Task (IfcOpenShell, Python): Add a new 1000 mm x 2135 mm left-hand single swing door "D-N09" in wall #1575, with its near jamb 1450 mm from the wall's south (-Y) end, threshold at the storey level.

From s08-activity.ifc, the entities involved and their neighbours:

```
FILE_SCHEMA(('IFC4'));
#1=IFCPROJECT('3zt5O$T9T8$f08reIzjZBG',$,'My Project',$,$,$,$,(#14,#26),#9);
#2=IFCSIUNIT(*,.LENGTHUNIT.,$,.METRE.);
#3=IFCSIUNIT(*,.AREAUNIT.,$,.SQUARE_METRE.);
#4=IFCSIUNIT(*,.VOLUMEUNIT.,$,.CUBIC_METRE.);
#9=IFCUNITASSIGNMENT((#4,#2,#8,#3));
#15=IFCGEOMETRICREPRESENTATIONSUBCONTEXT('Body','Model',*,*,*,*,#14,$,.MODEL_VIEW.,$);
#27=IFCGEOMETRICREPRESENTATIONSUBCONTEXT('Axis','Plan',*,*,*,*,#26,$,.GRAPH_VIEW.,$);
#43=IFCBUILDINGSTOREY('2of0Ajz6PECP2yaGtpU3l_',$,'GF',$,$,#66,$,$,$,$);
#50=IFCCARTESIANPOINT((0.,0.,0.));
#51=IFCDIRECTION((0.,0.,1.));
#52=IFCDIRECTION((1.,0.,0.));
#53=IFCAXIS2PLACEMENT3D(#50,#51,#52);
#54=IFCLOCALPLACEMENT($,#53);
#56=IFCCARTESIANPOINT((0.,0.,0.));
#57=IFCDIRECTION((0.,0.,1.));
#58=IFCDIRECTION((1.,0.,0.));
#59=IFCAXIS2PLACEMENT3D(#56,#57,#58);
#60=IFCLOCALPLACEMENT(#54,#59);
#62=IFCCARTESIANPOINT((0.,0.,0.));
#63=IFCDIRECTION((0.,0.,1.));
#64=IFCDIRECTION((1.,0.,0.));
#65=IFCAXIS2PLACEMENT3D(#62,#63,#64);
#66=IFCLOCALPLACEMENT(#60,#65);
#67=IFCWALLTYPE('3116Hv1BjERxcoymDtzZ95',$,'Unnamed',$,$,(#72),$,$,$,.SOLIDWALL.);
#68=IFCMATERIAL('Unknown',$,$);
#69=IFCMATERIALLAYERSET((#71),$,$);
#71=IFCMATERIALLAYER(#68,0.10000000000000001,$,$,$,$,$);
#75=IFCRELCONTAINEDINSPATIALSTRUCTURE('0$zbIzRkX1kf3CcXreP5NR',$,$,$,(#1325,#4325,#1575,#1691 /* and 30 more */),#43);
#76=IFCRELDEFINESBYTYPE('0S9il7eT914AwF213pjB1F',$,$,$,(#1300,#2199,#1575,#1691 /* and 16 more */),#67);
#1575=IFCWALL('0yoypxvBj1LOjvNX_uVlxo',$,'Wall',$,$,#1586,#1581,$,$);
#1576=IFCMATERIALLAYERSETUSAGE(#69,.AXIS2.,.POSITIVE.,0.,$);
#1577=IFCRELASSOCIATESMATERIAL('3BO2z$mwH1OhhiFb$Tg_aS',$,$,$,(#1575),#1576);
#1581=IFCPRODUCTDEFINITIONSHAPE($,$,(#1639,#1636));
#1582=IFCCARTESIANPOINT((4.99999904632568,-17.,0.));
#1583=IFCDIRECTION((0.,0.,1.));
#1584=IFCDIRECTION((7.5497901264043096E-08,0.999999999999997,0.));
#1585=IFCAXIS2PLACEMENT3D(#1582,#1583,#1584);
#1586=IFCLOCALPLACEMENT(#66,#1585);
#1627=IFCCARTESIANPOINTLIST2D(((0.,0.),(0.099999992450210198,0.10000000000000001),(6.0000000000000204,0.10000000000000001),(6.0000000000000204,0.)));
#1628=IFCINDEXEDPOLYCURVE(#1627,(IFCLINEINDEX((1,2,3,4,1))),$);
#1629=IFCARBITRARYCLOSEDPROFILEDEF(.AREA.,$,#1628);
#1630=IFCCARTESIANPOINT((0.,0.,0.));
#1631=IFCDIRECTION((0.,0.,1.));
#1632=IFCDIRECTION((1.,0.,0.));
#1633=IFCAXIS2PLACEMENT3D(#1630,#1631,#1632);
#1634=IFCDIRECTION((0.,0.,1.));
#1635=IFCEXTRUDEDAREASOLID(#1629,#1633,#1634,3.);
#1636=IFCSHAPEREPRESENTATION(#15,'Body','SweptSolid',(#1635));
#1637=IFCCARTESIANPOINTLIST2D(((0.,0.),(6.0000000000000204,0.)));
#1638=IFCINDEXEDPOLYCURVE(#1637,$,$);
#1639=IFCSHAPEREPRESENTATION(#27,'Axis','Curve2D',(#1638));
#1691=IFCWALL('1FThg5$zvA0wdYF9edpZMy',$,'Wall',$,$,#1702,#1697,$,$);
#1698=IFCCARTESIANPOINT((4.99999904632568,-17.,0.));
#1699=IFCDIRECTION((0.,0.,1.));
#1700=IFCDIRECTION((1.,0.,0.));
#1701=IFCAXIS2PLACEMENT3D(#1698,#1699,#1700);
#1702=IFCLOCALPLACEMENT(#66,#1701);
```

```python
import numpy as np
import ifcopenshell
import ifcopenshell.api.feature
import ifcopenshell.api.geometry
import ifcopenshell.api.root
import ifcopenshell.api.spatial
import ifcopenshell.geom
import ifcopenshell.util.element
import ifcopenshell.util.placement
import ifcopenshell.util.representation
import ifcopenshell.util.shape
import ifcopenshell.util.unit

model = ifcopenshell.open("s08-activity.ifc")
unit_scale = ifcopenshell.util.unit.calculate_unit_scale(model)
settings = ifcopenshell.geom.settings()


def volume(element):
    """Net volume in cubic metres, openings subtracted."""
    shape = ifcopenshell.geom.create_shape(settings, element)
    return ifcopenshell.util.shape.get_volume(shape.geometry)


wall = model.by_guid("0yoypxvBj1LOjvNX_uVlxo")
storey = ifcopenshell.util.element.get_container(wall, ifc_class="IfcBuildingStorey")
context = ifcopenshell.util.representation.get_context(model, "Model", "Body", "MODEL_VIEW")
before = volume(wall)

width, height, from_end, sill = 1, 2.135, 1.45, 0.0  # metres

# The wall runs along its own X axis, and the end named is its -X end.
wall_shape = ifcopenshell.geom.create_shape(settings, wall)
x, y, z = ifcopenshell.util.shape.get_vertices(wall_shape.geometry).T
start = x.min() + from_end
face, thickness = float(y.min()), float(y.max() - y.min())
wall_matrix = ifcopenshell.util.placement.get_local_placement(wall.ObjectPlacement)
level = ifcopenshell.util.placement.get_local_placement(storey.ObjectPlacement)[2, 3]


def in_wall(x, y):
    """Placement at x, y metres in the wall's axes, at sill height."""
    matrix = wall_matrix.copy()
    matrix[:, 3] = wall_matrix @ np.array([x / unit_scale, y / unit_scale, 0.0, 1.0])
    matrix[2, 3] = level + sill / unit_scale
    return matrix


# Opening: a box that overshoots both wall faces by 50 mm.
opening = ifcopenshell.api.root.create_entity(model, ifc_class="IfcOpeningElement", predefined_type="OPENING")
box = ifcopenshell.api.geometry.add_wall_representation(
    model, context=context, length=width, height=height, thickness=thickness + 0.1
)
ifcopenshell.api.geometry.assign_representation(model, product=opening, representation=box)
ifcopenshell.api.geometry.edit_object_placement(model, product=opening, matrix=in_wall(start, face - 0.05), is_si=False)
ifcopenshell.api.feature.add_feature(model, feature=opening, element=wall)

door = ifcopenshell.api.root.create_entity(model, ifc_class="IfcDoor", name="D-N09", predefined_type="DOOR")
door.OverallWidth, door.OverallHeight = width / unit_scale, height / unit_scale
door.OperationType = "SINGLE_SWING_LEFT"
body = ifcopenshell.api.geometry.add_door_representation(
    model,
    context=context,
    overall_width=door.OverallWidth,
    overall_height=door.OverallHeight,
    operation_type="SINGLE_SWING_LEFT",
    lining_properties={"LiningDepth": thickness / unit_scale, "ThresholdDepth": thickness / unit_scale},
)
ifcopenshell.api.geometry.assign_representation(model, product=door, representation=body)
ifcopenshell.api.spatial.assign_container(model, products=[door], relating_structure=storey)
ifcopenshell.api.feature.add_filling(model, opening=opening, element=door)

# The lining spans the wall, so the door starts at the wall face.
ifcopenshell.api.geometry.edit_object_placement(model, product=door, matrix=in_wall(start, face), is_si=False)

after = volume(wall)

print(f"wall volume {before:.3f} -> {after:.3f} m3")

model.write("s08-activity_edited.ifc")
```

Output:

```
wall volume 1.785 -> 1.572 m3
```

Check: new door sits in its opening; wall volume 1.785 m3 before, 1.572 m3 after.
